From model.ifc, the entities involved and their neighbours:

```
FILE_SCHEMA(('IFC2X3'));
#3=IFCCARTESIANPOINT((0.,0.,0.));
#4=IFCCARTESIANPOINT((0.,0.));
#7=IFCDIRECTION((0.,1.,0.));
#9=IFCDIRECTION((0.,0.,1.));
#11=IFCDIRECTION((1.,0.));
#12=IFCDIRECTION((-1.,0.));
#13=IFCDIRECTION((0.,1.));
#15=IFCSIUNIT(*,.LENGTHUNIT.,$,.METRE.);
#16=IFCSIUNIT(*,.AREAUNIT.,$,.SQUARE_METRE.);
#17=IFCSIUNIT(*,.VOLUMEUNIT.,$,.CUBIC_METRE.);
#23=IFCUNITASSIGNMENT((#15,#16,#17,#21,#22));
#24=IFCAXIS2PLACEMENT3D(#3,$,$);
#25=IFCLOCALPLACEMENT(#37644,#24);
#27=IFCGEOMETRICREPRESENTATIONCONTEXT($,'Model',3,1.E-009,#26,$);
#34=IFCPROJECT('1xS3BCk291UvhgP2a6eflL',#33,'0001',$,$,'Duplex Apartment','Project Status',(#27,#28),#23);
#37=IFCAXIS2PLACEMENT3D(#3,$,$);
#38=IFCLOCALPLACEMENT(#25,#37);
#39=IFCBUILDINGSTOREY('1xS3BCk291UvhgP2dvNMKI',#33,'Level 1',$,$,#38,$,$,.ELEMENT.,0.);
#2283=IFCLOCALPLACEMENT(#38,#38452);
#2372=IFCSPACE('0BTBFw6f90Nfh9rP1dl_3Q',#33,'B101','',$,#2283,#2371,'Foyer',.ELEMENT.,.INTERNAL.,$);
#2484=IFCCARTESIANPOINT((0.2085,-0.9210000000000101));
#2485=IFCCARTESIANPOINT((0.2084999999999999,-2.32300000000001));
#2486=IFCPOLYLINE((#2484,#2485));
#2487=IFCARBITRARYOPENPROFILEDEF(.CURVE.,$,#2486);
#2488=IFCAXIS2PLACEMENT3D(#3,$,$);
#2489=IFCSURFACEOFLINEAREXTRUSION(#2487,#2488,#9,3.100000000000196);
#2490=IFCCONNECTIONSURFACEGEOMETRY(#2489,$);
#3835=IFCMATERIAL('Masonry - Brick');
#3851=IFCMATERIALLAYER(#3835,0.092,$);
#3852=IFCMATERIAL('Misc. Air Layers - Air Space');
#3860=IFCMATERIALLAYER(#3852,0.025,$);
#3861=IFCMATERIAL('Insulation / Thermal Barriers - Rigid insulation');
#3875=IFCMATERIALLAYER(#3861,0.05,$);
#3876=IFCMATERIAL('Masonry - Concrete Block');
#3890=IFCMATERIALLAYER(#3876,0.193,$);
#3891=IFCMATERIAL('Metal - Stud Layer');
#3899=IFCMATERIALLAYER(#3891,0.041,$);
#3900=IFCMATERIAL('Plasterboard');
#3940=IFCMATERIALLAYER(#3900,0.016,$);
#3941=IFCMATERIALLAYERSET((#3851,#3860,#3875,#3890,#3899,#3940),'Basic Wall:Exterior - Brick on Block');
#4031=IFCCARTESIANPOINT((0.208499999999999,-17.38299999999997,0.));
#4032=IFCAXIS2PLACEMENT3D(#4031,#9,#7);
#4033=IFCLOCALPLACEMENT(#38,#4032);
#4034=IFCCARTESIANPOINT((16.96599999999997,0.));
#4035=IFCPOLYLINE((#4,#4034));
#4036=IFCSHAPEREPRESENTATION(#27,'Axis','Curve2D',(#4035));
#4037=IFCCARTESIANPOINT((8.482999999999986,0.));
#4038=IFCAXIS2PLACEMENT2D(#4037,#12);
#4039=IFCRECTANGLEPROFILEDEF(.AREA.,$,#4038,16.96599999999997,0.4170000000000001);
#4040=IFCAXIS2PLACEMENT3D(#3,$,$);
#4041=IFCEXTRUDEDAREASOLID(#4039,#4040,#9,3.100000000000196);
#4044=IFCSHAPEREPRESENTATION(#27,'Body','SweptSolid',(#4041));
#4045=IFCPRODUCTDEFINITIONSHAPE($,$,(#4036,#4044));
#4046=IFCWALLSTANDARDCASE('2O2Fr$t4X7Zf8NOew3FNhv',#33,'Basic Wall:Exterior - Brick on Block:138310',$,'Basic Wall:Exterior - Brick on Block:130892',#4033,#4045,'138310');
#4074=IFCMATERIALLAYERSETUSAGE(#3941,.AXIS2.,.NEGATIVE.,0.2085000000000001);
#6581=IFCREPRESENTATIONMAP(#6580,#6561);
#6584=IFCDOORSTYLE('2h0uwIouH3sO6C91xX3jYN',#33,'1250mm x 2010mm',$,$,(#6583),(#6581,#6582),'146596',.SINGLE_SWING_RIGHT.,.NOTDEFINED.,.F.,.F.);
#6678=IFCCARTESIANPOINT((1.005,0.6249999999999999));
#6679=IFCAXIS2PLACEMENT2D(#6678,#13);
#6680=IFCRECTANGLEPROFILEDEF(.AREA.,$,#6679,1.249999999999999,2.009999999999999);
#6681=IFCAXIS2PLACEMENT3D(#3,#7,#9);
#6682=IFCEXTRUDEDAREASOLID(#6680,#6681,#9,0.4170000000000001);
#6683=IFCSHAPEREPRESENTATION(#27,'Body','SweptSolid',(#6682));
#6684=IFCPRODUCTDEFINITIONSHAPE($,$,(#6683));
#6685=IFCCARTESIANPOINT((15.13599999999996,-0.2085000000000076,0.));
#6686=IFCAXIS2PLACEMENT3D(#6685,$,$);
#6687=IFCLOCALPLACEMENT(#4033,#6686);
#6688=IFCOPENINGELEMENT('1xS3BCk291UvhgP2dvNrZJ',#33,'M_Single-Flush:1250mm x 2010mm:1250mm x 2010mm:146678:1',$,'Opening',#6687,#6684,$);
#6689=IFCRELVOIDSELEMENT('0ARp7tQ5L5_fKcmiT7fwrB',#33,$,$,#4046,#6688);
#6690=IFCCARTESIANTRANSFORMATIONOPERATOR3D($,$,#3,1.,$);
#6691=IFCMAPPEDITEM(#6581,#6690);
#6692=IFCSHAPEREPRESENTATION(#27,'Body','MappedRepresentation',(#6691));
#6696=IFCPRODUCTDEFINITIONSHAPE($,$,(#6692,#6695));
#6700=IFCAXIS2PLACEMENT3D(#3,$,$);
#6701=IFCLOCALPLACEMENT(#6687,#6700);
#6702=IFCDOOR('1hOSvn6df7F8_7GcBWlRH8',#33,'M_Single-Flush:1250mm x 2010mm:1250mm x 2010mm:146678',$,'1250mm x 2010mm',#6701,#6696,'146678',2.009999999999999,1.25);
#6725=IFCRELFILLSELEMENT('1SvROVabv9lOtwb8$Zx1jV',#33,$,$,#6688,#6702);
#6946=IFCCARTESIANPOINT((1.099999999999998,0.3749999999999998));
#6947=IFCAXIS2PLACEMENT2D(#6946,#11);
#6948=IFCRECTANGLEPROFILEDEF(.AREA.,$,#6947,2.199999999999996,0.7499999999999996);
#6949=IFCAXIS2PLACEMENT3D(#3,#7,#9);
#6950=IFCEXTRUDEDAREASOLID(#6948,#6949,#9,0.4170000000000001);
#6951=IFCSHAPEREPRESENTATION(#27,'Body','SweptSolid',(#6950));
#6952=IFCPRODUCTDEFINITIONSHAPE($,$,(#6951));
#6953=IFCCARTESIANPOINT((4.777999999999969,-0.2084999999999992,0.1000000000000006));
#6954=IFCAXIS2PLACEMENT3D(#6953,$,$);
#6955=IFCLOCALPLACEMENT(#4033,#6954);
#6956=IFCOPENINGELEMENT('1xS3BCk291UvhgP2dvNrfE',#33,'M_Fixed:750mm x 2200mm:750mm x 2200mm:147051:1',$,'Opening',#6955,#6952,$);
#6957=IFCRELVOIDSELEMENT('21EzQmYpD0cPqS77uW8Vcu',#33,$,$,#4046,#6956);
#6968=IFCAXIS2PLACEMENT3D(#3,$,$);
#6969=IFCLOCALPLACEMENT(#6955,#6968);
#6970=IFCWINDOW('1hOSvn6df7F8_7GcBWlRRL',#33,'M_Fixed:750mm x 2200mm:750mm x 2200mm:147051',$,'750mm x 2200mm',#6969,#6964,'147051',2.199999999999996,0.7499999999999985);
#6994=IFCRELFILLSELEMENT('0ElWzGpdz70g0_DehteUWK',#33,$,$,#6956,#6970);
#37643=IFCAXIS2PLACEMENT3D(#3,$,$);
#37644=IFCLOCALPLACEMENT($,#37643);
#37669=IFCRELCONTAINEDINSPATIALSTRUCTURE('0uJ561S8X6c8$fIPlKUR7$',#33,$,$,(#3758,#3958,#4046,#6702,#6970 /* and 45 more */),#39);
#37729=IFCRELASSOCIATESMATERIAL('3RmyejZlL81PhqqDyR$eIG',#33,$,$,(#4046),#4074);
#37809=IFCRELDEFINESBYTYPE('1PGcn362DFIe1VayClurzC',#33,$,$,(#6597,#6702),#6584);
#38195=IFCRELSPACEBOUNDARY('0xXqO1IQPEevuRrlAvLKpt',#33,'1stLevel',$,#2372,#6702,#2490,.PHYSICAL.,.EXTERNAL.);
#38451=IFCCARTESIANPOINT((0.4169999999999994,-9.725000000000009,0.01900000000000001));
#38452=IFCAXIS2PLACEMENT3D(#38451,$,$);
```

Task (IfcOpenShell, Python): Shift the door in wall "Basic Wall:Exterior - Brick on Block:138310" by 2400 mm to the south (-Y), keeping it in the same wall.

```python
import numpy as np
import ifcopenshell
import ifcopenshell.api.geometry
import ifcopenshell.util.placement
import ifcopenshell.util.unit

model = ifcopenshell.open("model.ifc")
unit_scale = ifcopenshell.util.unit.calculate_unit_scale(model)

door = model.by_guid("1hOSvn6df7F8_7GcBWlRH8")
opening = door.FillsVoids[0].RelatingOpeningElement
wall = opening.VoidsElements[0].RelatingBuildingElement

wall_matrix = ifcopenshell.util.placement.get_local_placement(wall.ObjectPlacement)
shift = wall_matrix[:3, 0] * -2.4 / unit_scale
before = ifcopenshell.util.placement.get_local_placement(door.ObjectPlacement)[:3, 3].copy()

# The door is placed relative to its opening, so it follows when the opening moves.
matrix = ifcopenshell.util.placement.get_local_placement(opening.ObjectPlacement)
matrix[:3, 3] += shift
ifcopenshell.api.geometry.edit_object_placement(
    model, product=opening, matrix=matrix, is_si=False, should_transform_children=True
)

# Space boundary surfaces are stored in each space's coordinates; move them too.
for rel in door.ProvidesBoundaries:
    if not rel.ConnectionGeometry:
        continue
    surface = rel.ConnectionGeometry.SurfaceOnRelatingElement
    space_matrix = ifcopenshell.util.placement.get_local_placement(rel.RelatingSpace.ObjectPlacement)
    point = np.array(surface.Position.Location.Coordinates) + space_matrix[:3, :3].T @ shift
    surface.Position = model.createIfcAxis2Placement3D(
        model.createIfcCartesianPoint(point.tolist()), surface.Position.Axis, surface.Position.RefDirection
    )

after = ifcopenshell.util.placement.get_local_placement(door.ObjectPlacement)[:3, 3]
print("door moved by", (after - before).round(3) + 0.0)

model.write("model_edited.ifc")
```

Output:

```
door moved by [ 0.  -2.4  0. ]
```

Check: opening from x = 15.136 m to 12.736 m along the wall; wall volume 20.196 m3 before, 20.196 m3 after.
